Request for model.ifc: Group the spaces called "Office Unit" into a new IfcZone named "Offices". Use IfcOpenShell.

First a look at what the model holds.

```python
import ifcopenshell

model = ifcopenshell.open("model.ifc")
print(model.schema)
seen = {}
for space in model.by_type("IfcSpace"):
    seen[space.LongName] = seen.get(space.LongName, 0) + 1
for name, count in sorted(seen.items(), key=str):
    print(count, "x", name)
print("zones:", [z.Name for z in model.by_type("IfcZone")][:20])
```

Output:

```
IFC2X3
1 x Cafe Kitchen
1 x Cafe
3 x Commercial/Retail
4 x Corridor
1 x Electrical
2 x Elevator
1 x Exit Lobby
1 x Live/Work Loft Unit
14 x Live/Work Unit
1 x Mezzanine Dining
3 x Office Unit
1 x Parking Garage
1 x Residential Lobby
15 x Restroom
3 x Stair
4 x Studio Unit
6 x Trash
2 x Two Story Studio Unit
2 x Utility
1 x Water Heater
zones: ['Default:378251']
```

```python
import ifcopenshell
import ifcopenshell.api.group
import ifcopenshell.api.root

model = ifcopenshell.open("model.ifc")

names = {"Office Unit"}
spaces = [s for s in model.by_type("IfcSpace") if s.LongName in names]

zone = ifcopenshell.api.root.create_entity(model, ifc_class="IfcZone", name="Offices")
ifcopenshell.api.group.assign_group(model, products=spaces, group=zone)
print(len(spaces), "spaces in", zone.Name)

model.write("model_edited.ifc")
```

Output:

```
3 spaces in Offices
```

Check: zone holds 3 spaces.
